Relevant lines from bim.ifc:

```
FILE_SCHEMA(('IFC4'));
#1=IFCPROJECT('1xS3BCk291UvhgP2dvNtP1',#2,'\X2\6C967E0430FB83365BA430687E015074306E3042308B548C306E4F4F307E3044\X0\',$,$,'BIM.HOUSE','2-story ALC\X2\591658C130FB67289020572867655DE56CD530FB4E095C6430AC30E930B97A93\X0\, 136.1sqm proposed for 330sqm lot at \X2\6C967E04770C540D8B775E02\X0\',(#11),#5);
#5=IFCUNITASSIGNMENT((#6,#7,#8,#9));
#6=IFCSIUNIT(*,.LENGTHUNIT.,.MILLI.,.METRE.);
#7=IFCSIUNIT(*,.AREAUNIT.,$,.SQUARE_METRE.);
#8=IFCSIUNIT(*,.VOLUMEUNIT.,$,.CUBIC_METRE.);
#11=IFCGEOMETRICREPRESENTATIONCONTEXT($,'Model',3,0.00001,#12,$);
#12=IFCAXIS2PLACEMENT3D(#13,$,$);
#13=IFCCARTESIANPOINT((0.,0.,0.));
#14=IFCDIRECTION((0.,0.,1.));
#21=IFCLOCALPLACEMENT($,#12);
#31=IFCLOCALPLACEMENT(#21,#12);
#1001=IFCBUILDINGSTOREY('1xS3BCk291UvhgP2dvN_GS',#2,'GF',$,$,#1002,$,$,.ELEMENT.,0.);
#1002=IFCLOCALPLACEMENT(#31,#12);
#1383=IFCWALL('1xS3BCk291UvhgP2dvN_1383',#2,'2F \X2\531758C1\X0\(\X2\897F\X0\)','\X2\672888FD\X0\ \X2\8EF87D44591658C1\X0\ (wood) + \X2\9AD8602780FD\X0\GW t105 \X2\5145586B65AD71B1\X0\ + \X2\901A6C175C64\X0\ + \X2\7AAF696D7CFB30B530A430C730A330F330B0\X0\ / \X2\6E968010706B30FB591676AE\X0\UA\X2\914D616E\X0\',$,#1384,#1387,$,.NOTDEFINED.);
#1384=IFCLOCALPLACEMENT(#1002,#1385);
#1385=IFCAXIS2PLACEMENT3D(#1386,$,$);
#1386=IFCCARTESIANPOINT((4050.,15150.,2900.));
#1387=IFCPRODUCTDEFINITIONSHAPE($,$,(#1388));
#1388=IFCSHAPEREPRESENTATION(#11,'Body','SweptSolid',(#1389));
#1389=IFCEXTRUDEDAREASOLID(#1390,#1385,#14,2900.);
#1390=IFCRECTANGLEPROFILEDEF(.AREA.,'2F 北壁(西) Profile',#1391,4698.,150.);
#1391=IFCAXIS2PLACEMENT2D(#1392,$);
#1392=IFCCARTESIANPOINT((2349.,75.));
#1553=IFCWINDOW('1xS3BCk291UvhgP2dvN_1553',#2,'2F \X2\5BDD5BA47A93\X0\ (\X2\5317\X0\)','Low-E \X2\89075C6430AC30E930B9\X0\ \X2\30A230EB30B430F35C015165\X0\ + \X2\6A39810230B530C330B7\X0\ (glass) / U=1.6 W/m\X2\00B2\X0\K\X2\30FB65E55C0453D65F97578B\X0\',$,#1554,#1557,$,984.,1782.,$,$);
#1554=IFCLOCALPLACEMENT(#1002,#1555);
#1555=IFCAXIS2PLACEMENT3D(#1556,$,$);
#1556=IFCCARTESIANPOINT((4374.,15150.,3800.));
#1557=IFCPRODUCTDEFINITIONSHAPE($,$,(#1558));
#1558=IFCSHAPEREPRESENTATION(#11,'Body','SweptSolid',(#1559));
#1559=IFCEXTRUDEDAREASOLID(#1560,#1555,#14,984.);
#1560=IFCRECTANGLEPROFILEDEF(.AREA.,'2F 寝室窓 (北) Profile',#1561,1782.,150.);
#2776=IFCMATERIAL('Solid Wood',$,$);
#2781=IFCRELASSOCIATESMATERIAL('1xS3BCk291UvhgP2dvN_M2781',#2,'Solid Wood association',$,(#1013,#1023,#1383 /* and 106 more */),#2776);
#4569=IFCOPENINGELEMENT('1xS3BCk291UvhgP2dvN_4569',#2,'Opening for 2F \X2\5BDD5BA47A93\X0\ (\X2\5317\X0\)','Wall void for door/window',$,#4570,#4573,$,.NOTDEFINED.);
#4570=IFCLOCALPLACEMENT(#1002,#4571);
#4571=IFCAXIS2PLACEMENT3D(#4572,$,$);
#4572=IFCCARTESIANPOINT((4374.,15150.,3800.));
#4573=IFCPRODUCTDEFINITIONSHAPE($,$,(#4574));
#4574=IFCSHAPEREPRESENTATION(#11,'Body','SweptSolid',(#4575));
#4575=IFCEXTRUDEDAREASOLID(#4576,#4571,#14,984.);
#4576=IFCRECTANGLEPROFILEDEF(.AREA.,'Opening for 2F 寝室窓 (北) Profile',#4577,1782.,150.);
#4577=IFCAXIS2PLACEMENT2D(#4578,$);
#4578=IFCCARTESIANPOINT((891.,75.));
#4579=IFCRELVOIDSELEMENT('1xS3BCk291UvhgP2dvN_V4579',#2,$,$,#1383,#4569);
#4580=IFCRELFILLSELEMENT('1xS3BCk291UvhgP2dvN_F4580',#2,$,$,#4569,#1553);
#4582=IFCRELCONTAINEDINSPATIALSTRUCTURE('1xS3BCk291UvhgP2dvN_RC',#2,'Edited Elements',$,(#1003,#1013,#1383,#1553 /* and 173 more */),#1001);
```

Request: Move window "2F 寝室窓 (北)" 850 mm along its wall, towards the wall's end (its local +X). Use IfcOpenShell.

```python
import ifcopenshell
import ifcopenshell.api.geometry
import ifcopenshell.util.placement

model = ifcopenshell.open("bim.ifc")

window = model.by_id(1553)
opening = window.FillsVoids[0].RelatingOpeningElement
wall = opening.VoidsElements[0].RelatingBuildingElement

wall_matrix = ifcopenshell.util.placement.get_local_placement(wall.ObjectPlacement)
shift = wall_matrix[:3, 0] * 850.0
before = ifcopenshell.util.placement.get_local_placement(window.ObjectPlacement)[:3, 3].copy()

# The window is not placed relative to its opening, so move both.
for product in (opening, window):
    matrix = ifcopenshell.util.placement.get_local_placement(product.ObjectPlacement)
    matrix[:3, 3] += shift
    ifcopenshell.api.geometry.edit_object_placement(model, product=product, matrix=matrix, is_si=False)

after = ifcopenshell.util.placement.get_local_placement(window.ObjectPlacement)[:3, 3]
print("window moved by", (after - before).round(3) + 0.0)

model.write("bim_v2.ifc")
```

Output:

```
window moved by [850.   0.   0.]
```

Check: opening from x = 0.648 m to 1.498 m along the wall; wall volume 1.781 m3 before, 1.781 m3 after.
